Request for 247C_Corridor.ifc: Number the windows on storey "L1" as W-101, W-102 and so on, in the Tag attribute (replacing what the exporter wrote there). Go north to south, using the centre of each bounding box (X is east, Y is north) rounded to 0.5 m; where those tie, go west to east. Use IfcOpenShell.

First a look at what the model holds.

```python
import ifcopenshell
import ifcopenshell.util.element
import ifcopenshell.util.placement

model = ifcopenshell.open("247C_Corridor.ifc")
print(model.schema)
storey = next(s for s in model.by_type("IfcBuildingStorey") if s.Name == "L1")
windows = [e for e in ifcopenshell.util.element.get_decomposition(storey) if e.is_a("IfcWindow")]
for e in sorted(windows, key=lambda e: e.id()):
    origin = ifcopenshell.util.placement.get_local_placement(e.ObjectPlacement)[:3, 3]
    print(e.id(), e.Tag, e.Name, origin.round(2) + 0.0, sep=" | ")
```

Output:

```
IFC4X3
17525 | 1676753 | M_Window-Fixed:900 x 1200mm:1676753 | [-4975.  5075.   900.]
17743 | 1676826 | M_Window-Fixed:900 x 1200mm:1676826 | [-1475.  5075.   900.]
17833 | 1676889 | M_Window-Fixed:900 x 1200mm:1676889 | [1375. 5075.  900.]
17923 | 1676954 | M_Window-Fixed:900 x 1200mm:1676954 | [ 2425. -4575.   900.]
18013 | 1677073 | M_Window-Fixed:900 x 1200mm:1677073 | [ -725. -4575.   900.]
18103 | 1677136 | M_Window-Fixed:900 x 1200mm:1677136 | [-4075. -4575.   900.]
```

```python
import ifcopenshell
import ifcopenshell.geom
import ifcopenshell.util.element
import ifcopenshell.util.shape

model = ifcopenshell.open("247C_Corridor.ifc")
settings = ifcopenshell.geom.settings()
settings.set("use-world-coords", True)


def centre(element):
    shape = ifcopenshell.geom.create_shape(settings, element)
    return ifcopenshell.util.shape.get_bbox_centroid(shape.geometry)


storey = next(s for s in model.by_type("IfcBuildingStorey") if s.Name == "L1")
windows = [e for e in ifcopenshell.util.element.get_decomposition(storey) if e.is_a("IfcWindow")]

# Insertion points can sit at a corner or the storey origin, so sort by the geometry (in metres).
centres = {e: centre(e) for e in windows}
windows.sort(key=lambda e: (-round(centres[e][1] / 0.5), centres[e][0]))

for i, e in enumerate(windows, start=1):
    number = f"W-1{i:02d}"
    e.Tag = number
    print(e.id(), number)

model.write("247C_Corridor_edited.ifc")
```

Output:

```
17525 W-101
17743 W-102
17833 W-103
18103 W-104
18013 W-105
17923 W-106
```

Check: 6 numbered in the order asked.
